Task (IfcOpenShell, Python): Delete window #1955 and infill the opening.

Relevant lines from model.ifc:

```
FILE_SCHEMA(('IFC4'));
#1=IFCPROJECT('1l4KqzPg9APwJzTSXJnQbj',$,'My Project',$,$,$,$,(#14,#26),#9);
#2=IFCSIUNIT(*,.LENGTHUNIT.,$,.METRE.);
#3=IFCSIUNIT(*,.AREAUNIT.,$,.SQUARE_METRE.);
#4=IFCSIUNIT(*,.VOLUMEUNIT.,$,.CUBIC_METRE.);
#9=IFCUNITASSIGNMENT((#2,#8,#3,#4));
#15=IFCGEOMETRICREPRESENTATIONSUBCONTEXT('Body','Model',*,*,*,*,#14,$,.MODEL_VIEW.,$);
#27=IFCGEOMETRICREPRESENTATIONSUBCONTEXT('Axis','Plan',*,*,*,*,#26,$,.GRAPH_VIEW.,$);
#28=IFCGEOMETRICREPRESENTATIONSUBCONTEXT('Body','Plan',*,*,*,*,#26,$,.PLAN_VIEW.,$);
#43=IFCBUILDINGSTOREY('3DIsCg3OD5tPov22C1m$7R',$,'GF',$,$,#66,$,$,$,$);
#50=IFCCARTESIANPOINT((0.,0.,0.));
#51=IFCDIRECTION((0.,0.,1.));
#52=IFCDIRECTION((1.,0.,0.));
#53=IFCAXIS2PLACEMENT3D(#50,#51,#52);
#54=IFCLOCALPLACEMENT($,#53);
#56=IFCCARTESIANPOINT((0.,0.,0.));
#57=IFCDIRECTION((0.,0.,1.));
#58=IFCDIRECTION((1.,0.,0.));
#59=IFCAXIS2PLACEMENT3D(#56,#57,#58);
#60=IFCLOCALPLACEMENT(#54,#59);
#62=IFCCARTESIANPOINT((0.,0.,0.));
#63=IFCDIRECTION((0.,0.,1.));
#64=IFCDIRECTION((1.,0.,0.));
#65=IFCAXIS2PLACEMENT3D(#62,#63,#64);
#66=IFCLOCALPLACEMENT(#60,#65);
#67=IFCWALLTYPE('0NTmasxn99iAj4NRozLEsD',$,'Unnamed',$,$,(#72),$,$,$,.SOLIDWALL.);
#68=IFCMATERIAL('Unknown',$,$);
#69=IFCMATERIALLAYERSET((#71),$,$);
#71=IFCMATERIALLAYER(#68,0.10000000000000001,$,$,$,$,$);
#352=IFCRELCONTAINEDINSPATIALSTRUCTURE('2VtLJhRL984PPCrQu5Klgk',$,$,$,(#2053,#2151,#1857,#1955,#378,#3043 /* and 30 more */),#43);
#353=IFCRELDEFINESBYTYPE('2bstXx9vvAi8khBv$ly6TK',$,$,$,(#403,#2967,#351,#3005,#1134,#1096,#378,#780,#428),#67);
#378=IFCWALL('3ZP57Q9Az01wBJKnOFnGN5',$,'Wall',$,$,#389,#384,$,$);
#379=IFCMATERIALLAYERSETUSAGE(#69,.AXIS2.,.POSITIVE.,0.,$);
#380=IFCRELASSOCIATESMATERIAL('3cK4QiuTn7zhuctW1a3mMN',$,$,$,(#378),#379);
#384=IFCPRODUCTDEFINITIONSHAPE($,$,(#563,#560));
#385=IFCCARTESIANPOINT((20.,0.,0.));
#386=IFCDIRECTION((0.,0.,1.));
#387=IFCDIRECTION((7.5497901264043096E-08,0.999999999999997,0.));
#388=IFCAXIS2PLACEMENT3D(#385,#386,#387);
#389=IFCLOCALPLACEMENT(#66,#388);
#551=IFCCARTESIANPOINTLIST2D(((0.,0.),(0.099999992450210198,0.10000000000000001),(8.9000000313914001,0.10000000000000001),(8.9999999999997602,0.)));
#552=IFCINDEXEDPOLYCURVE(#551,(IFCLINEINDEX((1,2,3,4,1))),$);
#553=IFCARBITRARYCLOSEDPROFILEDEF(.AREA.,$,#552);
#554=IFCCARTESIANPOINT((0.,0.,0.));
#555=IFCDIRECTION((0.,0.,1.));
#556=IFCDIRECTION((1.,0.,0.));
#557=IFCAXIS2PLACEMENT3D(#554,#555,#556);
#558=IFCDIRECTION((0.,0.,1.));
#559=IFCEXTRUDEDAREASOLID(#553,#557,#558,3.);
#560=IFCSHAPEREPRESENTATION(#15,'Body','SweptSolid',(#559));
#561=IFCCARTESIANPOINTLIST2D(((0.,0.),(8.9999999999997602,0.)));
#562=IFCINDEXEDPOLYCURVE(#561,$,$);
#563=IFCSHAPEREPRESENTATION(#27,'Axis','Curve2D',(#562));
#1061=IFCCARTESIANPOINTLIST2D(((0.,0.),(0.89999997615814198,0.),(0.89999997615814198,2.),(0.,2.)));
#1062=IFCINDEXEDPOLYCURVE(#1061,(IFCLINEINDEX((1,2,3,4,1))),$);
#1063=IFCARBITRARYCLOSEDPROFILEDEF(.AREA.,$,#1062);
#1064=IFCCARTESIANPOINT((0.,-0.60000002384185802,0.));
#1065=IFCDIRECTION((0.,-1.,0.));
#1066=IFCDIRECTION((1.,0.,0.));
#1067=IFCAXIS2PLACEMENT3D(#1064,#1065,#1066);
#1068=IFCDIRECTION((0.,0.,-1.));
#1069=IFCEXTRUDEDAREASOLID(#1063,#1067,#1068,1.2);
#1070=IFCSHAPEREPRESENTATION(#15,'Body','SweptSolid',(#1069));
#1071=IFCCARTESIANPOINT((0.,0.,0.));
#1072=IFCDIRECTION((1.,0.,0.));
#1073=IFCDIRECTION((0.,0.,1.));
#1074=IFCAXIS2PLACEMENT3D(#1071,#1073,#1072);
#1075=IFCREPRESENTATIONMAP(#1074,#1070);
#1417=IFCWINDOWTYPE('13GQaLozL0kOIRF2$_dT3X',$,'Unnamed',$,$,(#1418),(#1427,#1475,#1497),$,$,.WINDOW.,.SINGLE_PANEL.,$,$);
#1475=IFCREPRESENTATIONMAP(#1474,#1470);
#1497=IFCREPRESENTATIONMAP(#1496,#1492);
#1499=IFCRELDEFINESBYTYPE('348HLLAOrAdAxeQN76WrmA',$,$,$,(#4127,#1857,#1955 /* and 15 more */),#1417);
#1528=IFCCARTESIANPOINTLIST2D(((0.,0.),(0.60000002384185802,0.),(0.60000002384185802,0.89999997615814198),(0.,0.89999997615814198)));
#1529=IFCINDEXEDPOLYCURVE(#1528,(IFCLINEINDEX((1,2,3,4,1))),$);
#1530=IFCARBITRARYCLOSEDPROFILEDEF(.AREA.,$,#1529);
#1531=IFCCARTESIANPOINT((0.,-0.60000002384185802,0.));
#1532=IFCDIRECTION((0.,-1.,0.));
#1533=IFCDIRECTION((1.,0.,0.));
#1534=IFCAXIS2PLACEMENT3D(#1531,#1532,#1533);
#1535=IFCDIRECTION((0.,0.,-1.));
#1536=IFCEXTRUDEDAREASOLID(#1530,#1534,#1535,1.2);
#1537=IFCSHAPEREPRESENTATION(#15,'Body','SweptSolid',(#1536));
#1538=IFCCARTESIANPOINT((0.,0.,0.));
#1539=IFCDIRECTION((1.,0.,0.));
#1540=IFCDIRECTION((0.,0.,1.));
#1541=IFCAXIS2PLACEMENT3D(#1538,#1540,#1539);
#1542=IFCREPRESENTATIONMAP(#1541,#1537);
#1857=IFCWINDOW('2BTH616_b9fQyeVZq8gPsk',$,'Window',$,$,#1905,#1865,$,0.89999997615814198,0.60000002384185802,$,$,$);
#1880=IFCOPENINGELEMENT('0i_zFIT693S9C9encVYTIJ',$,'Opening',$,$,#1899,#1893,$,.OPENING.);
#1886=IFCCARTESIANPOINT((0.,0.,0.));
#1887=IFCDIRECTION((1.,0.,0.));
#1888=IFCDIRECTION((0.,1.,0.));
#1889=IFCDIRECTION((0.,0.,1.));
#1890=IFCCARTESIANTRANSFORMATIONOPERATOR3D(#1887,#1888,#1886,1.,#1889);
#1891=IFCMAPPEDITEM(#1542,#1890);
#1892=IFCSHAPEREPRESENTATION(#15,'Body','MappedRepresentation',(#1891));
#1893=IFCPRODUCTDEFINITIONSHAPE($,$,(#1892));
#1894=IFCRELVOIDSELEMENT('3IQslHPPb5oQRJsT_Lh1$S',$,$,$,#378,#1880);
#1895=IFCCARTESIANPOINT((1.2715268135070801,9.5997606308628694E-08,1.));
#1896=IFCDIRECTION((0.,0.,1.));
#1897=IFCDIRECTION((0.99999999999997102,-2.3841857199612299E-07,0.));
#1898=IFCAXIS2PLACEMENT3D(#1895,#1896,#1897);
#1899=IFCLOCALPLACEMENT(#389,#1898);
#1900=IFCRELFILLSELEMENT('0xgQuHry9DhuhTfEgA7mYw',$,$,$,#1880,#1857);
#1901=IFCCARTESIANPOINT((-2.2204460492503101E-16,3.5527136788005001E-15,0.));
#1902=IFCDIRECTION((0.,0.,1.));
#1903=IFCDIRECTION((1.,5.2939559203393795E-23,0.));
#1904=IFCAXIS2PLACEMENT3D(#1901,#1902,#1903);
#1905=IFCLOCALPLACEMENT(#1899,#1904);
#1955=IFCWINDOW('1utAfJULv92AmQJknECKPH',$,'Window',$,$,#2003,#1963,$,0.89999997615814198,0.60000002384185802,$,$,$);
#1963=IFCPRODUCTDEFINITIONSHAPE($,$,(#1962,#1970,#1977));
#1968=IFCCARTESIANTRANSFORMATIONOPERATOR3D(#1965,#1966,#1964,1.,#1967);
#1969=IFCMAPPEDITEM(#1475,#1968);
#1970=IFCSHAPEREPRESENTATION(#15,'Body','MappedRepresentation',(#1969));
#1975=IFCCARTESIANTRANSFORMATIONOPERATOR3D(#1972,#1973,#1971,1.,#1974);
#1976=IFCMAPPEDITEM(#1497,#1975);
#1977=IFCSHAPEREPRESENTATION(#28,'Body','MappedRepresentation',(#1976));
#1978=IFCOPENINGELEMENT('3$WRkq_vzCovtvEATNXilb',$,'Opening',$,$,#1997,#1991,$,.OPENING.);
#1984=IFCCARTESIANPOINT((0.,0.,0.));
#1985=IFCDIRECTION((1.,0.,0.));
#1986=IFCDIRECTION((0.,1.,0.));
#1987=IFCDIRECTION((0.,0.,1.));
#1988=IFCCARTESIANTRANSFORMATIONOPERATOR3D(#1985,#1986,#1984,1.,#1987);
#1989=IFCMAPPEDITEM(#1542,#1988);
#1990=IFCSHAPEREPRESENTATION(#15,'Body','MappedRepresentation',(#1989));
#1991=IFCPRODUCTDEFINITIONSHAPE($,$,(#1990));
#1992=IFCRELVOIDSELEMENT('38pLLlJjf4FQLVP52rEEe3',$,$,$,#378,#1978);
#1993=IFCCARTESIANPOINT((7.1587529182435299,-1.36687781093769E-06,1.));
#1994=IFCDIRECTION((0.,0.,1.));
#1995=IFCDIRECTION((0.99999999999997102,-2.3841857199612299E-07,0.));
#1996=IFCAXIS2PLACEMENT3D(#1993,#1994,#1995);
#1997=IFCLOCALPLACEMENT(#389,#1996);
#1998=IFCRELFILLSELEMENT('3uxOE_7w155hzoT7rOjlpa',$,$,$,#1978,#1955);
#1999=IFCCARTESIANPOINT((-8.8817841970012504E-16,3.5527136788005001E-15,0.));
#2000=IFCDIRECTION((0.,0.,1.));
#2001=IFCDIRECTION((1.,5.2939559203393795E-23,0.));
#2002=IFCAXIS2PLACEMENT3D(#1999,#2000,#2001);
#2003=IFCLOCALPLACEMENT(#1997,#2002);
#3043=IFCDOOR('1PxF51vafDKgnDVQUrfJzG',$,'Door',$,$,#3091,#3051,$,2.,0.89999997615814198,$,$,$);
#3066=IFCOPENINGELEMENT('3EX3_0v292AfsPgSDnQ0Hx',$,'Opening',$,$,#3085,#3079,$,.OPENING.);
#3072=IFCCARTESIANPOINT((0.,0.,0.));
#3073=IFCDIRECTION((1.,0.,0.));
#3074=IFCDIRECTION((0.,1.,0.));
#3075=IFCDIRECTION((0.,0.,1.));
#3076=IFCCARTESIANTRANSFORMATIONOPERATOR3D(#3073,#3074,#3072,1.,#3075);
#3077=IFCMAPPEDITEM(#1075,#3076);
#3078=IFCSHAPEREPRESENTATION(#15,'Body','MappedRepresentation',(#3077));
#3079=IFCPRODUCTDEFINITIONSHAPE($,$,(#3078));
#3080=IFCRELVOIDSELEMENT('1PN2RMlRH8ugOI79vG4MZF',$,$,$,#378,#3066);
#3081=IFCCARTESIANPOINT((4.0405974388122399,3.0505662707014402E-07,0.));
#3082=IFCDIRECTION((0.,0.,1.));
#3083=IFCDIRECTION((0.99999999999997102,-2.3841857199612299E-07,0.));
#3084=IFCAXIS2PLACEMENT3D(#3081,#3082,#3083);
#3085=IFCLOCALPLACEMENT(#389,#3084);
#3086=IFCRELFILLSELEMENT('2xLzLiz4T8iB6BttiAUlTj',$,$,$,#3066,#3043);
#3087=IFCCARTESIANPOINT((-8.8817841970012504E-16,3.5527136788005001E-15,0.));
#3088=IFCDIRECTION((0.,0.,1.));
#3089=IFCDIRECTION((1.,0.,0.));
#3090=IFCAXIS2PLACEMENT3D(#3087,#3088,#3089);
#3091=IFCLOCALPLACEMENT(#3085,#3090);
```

```python
import ifcopenshell
import ifcopenshell.api.feature
import ifcopenshell.api.root
import ifcopenshell.geom
import ifcopenshell.util.shape

model = ifcopenshell.open("model.ifc")
settings = ifcopenshell.geom.settings()


def volume(element):
    """Net volume in cubic metres, openings subtracted."""
    shape = ifcopenshell.geom.create_shape(settings, element)
    return ifcopenshell.util.shape.get_volume(shape.geometry)


window = model.by_guid("1utAfJULv92AmQJknECKPH")
opening = window.FillsVoids[0].RelatingOpeningElement
wall = opening.VoidsElements[0].RelatingBuildingElement
before = volume(wall)

ifcopenshell.api.root.remove_product(model, product=window)
ifcopenshell.api.feature.remove_feature(model, feature=opening)

after = volume(wall)

print(f"wall volume {before:.3f} -> {after:.3f} m3")

model.write("model_rev.ifc")
```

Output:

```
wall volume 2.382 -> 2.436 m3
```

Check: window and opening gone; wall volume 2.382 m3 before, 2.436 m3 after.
